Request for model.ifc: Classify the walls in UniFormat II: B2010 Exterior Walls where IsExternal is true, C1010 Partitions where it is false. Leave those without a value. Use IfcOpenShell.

First a look at what the model holds.

```python
import ifcopenshell
import ifcopenshell.util.element

model = ifcopenshell.open("model.ifc")
print(model.schema)
print("classifications:", [c.Name for c in model.by_type("IfcClassification")])
values = [ifcopenshell.util.element.get_pset(e, "Pset_WallCommon", "IsExternal") for e in model.by_type("IfcWall")]
for value in (True, False, None):
    print("IsExternal", value, values.count(value))
```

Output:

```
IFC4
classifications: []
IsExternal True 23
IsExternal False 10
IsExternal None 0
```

```python
import ifcopenshell
import ifcopenshell.api.classification
import ifcopenshell.util.element

model = ifcopenshell.open("model.ifc")

system = ifcopenshell.api.classification.add_classification(model, classification="UniFormat II")

walls = model.by_type("IfcWall")
external = {e: ifcopenshell.util.element.get_pset(e, "Pset_WallCommon", "IsExternal") for e in walls}
for flag, code, name in ((True, "B2010", "Exterior Walls"), (False, "C1010", "Partitions")):
    products = [e for e in walls if external[e] is flag]
    ifcopenshell.api.classification.add_reference(
        model, products=products, classification=system, identification=code, name=name
    )
    print(code, len(products))

model.write("model-out.ifc")
```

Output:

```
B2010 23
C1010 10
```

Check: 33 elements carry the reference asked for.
